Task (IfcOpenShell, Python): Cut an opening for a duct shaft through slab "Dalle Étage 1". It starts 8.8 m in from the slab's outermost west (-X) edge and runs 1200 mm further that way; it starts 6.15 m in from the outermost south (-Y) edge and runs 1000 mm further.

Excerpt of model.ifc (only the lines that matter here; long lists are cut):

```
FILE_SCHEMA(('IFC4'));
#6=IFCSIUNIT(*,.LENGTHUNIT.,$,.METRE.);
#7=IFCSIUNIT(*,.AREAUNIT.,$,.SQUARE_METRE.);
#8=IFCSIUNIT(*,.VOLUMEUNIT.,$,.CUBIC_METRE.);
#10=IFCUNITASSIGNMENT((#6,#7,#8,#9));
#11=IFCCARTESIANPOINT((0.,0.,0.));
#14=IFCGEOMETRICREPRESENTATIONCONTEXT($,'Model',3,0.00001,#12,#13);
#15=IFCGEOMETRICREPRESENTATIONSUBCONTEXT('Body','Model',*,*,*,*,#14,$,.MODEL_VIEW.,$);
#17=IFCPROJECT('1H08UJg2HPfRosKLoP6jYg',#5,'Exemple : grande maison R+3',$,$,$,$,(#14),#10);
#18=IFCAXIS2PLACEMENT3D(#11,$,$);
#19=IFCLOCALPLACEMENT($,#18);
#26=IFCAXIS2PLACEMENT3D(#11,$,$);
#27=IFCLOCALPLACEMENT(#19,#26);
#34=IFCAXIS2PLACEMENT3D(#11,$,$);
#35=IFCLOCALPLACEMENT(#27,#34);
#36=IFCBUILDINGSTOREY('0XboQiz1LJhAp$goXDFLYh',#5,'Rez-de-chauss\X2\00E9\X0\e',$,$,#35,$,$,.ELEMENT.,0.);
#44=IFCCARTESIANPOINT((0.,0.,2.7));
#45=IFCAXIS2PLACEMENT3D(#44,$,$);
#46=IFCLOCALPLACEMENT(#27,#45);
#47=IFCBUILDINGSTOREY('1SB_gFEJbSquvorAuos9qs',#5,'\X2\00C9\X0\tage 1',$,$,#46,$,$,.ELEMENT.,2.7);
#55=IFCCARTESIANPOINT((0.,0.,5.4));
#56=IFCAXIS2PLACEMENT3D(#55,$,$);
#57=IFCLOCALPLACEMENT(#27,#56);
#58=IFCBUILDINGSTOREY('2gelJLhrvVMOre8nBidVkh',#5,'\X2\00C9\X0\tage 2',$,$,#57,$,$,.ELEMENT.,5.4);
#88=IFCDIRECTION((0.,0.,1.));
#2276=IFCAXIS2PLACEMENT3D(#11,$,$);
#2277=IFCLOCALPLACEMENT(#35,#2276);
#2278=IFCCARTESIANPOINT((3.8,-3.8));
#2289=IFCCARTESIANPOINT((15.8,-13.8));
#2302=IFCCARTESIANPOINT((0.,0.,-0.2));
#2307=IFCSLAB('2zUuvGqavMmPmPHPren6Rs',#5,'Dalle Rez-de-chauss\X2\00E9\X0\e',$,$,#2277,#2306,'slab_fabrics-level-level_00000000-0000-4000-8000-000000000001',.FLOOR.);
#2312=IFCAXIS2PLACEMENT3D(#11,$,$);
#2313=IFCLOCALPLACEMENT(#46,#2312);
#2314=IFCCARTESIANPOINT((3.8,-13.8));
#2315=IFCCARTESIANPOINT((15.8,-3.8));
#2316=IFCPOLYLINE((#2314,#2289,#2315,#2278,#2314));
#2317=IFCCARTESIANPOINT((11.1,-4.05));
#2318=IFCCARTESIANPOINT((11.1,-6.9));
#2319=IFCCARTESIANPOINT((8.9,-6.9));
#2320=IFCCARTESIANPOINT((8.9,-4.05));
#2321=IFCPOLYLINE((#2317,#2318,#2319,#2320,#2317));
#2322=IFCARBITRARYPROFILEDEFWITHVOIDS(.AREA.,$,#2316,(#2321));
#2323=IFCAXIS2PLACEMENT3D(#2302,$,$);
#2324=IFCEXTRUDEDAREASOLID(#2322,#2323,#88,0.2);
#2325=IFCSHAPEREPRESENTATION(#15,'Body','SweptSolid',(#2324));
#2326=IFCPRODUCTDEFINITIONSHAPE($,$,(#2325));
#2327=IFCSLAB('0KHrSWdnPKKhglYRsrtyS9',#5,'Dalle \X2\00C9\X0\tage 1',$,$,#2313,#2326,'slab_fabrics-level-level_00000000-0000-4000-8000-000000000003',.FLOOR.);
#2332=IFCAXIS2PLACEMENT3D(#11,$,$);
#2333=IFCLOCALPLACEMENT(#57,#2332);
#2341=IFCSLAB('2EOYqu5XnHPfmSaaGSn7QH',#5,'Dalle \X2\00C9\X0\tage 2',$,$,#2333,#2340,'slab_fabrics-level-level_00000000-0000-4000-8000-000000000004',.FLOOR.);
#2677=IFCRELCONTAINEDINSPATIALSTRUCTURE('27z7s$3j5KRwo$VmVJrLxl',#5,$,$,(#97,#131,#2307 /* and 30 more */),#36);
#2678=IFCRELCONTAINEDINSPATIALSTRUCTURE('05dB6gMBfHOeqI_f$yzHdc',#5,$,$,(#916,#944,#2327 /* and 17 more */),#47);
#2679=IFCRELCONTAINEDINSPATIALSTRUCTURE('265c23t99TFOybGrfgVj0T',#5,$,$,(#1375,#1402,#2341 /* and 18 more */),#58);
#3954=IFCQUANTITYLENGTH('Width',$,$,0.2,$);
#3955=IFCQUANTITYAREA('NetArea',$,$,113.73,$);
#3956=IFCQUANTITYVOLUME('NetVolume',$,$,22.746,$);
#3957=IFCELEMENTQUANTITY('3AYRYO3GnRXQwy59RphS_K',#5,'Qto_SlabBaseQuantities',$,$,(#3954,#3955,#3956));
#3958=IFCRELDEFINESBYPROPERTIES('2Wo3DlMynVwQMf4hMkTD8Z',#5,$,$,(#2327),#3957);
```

```python
import numpy as np
import ifcopenshell
import ifcopenshell.api.feature
import ifcopenshell.api.geometry
import ifcopenshell.api.pset
import ifcopenshell.api.root
import ifcopenshell.geom
import ifcopenshell.util.element
import ifcopenshell.util.placement
import ifcopenshell.util.representation
import ifcopenshell.util.shape
import ifcopenshell.util.unit

model = ifcopenshell.open("model.ifc")
unit_scale = ifcopenshell.util.unit.calculate_unit_scale(model)
area_scale = ifcopenshell.util.unit.calculate_unit_scale(model, "AREAUNIT")
volume_scale = ifcopenshell.util.unit.calculate_unit_scale(model, "VOLUMEUNIT")
settings = ifcopenshell.geom.settings()


def volume(element):
    """Net volume in cubic metres, openings subtracted."""
    shape = ifcopenshell.geom.create_shape(settings, element)
    return ifcopenshell.util.shape.get_volume(shape.geometry)


slab = model.by_guid("0KHrSWdnPKKhglYRsrtyS9")
before = volume(slab)

# Extent in the slab's own axes, in metres. The edges named are its -X and -Y sides.
slab_shape = ifcopenshell.geom.create_shape(settings, slab)
vertices = ifcopenshell.util.shape.get_vertices(slab_shape.geometry)
x_min, y_min, bottom = vertices.min(axis=0)
top = vertices[:, 2].max()

opening = ifcopenshell.api.root.create_entity(model, ifc_class="IfcOpeningElement", name="Duct shaft opening", predefined_type="OPENING")
context = ifcopenshell.util.representation.get_context(model, "Model", "Body", "MODEL_VIEW")
width, depth = 1.2, 1
outline = [(0.0, 0.0), (width, 0.0), (width, depth), (0.0, depth), (0.0, 0.0)]
# Overshoot both faces by 50 mm so the cut is clean.
shape = ifcopenshell.api.geometry.add_slab_representation(
    model, context=context, depth=top - bottom + 0.1, polyline=outline
)
ifcopenshell.api.geometry.assign_representation(model, product=opening, representation=shape)

matrix = ifcopenshell.util.placement.get_local_placement(slab.ObjectPlacement)
matrix[:, 3] = matrix @ np.append(np.array([x_min + 8.8, y_min + 6.15, bottom - 0.05]) / unit_scale, 1.0)
ifcopenshell.api.geometry.edit_object_placement(model, product=opening, matrix=matrix, is_si=False)
ifcopenshell.api.feature.add_feature(model, feature=opening, element=slab)

after = volume(slab)

# Update the slab's stored quantities.
qto = model.by_id(ifcopenshell.util.element.get_pset(slab, "Qto_SlabBaseQuantities", should_inherit=False)["id"])
ifcopenshell.api.pset.edit_qto(model, qto=qto, properties={
    "NetArea": after / (top - bottom) / area_scale,
    "NetVolume": after / volume_scale,
})

print(f"slab volume {before:.3f} -> {after:.3f} m3")

model.write("model_v2.ifc")
```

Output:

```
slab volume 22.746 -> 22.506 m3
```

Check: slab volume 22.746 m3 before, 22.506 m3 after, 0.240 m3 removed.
